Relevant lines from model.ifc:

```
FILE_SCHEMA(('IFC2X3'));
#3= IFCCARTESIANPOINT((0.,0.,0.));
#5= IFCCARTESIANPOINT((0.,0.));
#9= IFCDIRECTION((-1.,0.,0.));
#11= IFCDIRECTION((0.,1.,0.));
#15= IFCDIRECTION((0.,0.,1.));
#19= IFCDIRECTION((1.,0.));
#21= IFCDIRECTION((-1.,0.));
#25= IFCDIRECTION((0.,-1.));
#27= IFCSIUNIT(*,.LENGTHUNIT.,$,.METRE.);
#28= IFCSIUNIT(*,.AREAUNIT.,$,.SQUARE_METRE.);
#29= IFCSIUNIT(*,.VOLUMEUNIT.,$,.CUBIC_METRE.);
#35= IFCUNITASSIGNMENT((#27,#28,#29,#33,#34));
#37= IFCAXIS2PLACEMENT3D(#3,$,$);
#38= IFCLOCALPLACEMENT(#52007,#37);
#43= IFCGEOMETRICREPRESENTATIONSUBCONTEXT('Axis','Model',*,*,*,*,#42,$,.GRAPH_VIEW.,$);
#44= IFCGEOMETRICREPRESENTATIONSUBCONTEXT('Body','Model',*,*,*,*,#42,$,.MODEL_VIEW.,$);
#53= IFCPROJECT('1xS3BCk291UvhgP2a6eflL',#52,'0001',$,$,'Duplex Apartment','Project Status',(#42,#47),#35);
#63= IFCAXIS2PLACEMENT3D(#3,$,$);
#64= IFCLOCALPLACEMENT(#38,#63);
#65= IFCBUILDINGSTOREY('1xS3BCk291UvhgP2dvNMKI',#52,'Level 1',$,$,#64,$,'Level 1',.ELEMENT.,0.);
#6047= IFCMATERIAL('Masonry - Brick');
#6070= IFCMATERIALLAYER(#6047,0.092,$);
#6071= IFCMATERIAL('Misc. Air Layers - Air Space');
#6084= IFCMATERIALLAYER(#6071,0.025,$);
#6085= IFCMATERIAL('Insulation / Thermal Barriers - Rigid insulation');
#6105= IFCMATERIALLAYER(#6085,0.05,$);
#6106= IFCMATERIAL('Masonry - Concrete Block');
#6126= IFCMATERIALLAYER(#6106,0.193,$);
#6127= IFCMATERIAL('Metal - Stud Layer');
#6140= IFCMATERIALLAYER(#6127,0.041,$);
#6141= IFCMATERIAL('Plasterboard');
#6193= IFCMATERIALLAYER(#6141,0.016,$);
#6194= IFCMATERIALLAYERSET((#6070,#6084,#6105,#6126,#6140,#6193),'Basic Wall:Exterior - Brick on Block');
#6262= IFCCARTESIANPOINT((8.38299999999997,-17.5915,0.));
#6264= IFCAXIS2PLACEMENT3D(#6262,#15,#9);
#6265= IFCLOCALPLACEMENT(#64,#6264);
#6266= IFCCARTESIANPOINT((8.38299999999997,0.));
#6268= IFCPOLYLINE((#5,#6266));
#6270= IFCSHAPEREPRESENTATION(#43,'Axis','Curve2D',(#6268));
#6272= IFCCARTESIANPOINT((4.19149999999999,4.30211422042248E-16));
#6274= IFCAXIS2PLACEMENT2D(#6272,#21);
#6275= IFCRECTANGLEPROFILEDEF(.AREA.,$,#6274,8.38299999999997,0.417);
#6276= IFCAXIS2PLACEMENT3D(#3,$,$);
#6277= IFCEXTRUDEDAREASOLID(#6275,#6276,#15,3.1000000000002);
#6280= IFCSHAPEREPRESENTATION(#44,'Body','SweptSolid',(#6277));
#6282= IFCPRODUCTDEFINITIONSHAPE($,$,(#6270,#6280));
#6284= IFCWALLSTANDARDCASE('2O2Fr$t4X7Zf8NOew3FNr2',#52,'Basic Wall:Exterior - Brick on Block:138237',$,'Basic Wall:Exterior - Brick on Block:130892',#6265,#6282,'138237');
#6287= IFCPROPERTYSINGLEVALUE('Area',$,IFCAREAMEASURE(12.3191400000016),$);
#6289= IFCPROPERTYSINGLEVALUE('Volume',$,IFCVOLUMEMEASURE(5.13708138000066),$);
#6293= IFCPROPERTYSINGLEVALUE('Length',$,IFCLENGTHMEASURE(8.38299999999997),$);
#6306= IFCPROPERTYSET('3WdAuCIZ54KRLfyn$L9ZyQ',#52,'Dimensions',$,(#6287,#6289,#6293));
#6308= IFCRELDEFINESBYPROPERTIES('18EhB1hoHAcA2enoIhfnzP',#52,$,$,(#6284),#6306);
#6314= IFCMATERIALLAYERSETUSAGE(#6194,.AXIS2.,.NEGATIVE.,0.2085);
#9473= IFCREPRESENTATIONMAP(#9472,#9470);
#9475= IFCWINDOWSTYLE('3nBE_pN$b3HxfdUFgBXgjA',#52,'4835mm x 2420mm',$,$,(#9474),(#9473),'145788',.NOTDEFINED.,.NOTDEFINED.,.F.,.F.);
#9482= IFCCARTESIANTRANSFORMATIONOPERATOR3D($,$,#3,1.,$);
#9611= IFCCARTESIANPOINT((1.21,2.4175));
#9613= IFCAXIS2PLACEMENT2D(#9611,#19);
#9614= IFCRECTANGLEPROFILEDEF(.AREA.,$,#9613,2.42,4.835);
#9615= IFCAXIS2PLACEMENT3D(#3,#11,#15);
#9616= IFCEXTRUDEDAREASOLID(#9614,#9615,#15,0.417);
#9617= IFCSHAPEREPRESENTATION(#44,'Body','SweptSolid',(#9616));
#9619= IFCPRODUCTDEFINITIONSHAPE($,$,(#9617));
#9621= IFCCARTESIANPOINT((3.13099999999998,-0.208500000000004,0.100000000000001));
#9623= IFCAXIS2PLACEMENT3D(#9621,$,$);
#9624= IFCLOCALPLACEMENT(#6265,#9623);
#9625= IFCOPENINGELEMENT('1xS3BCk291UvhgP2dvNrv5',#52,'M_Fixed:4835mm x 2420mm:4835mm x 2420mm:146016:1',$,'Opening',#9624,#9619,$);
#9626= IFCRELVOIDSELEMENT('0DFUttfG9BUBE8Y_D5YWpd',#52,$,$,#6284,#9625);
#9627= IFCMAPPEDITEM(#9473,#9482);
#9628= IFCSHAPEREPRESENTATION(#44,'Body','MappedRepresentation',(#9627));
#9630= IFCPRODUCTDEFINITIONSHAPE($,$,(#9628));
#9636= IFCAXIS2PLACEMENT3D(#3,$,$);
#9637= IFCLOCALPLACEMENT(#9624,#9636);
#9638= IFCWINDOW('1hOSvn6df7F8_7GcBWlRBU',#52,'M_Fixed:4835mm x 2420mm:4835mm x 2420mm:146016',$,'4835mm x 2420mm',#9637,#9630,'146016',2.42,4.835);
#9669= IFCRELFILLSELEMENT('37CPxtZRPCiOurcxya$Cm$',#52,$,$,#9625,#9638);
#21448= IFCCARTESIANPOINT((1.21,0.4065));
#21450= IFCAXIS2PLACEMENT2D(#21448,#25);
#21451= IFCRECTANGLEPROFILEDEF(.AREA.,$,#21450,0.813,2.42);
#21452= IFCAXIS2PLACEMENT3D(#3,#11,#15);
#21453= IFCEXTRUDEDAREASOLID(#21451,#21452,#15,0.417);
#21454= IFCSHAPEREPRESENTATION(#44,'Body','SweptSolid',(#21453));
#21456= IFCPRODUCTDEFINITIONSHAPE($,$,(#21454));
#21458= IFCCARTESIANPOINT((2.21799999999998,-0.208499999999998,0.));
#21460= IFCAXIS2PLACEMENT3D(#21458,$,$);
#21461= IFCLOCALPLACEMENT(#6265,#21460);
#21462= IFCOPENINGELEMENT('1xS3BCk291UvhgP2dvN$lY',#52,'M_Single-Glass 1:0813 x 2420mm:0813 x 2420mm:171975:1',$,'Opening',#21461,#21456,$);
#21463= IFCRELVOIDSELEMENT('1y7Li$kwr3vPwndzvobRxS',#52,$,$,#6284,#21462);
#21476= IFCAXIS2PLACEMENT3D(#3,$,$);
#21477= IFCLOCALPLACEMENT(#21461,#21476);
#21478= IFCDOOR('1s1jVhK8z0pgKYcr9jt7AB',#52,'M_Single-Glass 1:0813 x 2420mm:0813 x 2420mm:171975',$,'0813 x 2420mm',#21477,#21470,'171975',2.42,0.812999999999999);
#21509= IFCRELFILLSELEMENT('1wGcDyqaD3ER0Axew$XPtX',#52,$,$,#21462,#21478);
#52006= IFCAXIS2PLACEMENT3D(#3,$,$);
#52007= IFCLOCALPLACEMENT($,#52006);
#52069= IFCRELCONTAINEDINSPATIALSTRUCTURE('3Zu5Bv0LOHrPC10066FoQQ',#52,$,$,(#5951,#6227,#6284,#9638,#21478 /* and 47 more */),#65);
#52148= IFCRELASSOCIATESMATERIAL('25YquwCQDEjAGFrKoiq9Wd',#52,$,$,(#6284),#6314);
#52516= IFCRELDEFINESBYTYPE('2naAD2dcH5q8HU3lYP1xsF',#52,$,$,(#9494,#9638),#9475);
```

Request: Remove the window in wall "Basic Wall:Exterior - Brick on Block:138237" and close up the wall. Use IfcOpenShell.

```python
import ifcopenshell
import ifcopenshell.api.feature
import ifcopenshell.api.pset
import ifcopenshell.api.root
import ifcopenshell.geom
import ifcopenshell.util.element
import ifcopenshell.util.shape
import ifcopenshell.util.unit

model = ifcopenshell.open("model.ifc")
area_scale = ifcopenshell.util.unit.calculate_unit_scale(model, "AREAUNIT")
volume_scale = ifcopenshell.util.unit.calculate_unit_scale(model, "VOLUMEUNIT")
settings = ifcopenshell.geom.settings()


def volume(element):
    """Net volume in cubic metres, openings subtracted."""
    shape = ifcopenshell.geom.create_shape(settings, element)
    return ifcopenshell.util.shape.get_volume(shape.geometry)


window = model.by_id(9638)
opening = window.FillsVoids[0].RelatingOpeningElement
wall = opening.VoidsElements[0].RelatingBuildingElement
before = volume(wall)

ifcopenshell.api.root.remove_product(model, product=window)
ifcopenshell.api.feature.remove_feature(model, feature=opening)

after = volume(wall)
thickness = 0.417  # wall thickness in metres

# Update the wall's stored quantities.
pset = model.by_id(ifcopenshell.util.element.get_pset(wall, "Dimensions", should_inherit=False)["id"])
ifcopenshell.api.pset.edit_pset(model, pset=pset, properties={
    "Area": model.create_entity("IfcAreaMeasure", after / thickness / area_scale),
    "Volume": model.create_entity("IfcVolumeMeasure", after / volume_scale),
})

print(f"wall volume {before:.3f} -> {after:.3f} m3")

model.write("model-out.ifc")
```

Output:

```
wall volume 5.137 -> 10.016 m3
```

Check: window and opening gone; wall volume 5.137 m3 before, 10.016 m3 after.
